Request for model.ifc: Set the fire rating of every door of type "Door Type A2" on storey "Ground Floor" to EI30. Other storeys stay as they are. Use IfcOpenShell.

First a look at what the model holds.

```python
import ifcopenshell
import ifcopenshell.util.element

model = ifcopenshell.open("model.ifc")
print(model.schema)
storey = next(s for s in model.by_type("IfcBuildingStorey") if s.Name == "Ground Floor")
doors = [e for e in ifcopenshell.util.element.get_decomposition(storey) if e.is_a("IfcDoor")]
seen = {}
for e in doors:
    element_type = ifcopenshell.util.element.get_type(e)
    key = (element_type.Name if element_type != e and element_type else None, ifcopenshell.util.element.get_pset(e, "Pset_DoorCommon", "FireRating"))
    seen[key] = seen.get(key, 0) + 1
for (name, value), count in sorted(seen.items(), key=str):
    print(count, "x", name, "|", value)
```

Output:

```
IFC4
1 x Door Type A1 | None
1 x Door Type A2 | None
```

```python
import ifcopenshell
import ifcopenshell.api.pset
import ifcopenshell.util.element

model = ifcopenshell.open("model.ifc")

storey = next(s for s in model.by_type("IfcBuildingStorey") if s.Name == "Ground Floor")
doors = [e for e in ifcopenshell.util.element.get_decomposition(storey) if e.is_a("IfcDoor")]

count = 0
for e in doors:
    element_type = ifcopenshell.util.element.get_type(e)
    if element_type in (None, e) or element_type.Name != "Door Type A2":
        continue
    # add_pset returns the element's existing set when there is one.
    pset = ifcopenshell.api.pset.add_pset(model, product=e, name="Pset_DoorCommon")
    ifcopenshell.api.pset.edit_pset(model, pset=pset, properties={"FireRating": "EI30"})
    count += 1

print(count, "doors updated")

model.write("model_updated.ifc")
```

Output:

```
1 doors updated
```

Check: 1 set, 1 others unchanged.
